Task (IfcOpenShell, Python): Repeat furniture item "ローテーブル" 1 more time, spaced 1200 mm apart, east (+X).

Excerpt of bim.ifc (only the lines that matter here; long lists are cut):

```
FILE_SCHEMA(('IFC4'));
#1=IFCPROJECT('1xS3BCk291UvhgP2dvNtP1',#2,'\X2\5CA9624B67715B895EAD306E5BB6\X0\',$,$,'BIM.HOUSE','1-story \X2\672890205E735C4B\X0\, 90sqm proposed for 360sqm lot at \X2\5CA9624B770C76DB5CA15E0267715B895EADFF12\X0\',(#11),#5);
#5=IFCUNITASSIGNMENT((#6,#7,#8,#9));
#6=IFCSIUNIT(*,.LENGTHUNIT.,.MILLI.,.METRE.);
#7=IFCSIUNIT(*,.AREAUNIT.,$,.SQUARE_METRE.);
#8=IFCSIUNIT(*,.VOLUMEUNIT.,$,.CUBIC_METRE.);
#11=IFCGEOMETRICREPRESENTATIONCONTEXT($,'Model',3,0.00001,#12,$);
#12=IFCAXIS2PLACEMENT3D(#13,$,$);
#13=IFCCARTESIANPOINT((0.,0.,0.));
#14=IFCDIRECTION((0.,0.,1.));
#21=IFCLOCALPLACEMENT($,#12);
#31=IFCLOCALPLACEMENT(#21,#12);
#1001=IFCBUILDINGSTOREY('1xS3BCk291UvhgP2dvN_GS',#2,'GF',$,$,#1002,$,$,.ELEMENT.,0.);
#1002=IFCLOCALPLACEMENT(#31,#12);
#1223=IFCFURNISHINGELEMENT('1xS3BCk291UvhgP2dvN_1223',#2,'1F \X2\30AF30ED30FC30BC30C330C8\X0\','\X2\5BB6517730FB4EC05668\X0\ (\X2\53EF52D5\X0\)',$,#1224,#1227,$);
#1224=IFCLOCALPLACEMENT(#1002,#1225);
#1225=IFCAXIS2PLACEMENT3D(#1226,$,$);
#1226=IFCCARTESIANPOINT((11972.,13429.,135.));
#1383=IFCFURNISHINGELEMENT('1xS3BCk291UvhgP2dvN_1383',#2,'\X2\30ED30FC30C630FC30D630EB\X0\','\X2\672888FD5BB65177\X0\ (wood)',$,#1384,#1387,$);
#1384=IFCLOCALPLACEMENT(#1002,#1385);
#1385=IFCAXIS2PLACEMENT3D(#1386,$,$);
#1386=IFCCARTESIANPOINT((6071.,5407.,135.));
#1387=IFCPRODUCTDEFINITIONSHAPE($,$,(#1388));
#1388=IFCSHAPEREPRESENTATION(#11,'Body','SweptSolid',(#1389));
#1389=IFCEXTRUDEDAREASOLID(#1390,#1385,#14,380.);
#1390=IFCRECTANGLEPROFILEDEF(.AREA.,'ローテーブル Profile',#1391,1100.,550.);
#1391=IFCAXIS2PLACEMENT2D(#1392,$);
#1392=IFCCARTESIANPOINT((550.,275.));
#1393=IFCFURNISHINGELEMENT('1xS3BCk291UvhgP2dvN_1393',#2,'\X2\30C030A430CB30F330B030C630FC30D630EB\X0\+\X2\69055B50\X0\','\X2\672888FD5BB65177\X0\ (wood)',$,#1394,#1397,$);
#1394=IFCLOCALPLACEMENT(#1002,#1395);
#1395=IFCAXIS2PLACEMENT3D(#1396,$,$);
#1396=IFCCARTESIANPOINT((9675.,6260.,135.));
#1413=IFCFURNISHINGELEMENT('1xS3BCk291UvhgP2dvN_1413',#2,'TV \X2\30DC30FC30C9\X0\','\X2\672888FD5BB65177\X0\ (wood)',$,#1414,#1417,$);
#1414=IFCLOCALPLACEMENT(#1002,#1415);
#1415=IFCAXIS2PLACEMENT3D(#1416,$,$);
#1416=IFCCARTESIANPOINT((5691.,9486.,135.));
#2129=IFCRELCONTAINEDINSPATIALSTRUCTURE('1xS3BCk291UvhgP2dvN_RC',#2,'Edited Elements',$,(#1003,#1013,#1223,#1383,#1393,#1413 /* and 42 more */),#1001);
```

```python
import numpy as np
import ifcopenshell
import ifcopenshell.api.geometry
import ifcopenshell.api.root
import ifcopenshell.util.element
import ifcopenshell.util.placement
import ifcopenshell.util.unit

model = ifcopenshell.open("bim.ifc")
unit_scale = ifcopenshell.util.unit.calculate_unit_scale(model)


def reuse_history(source, copy):
    """copy_class also copies each property set's owner history, people and application; keep the originals."""
    for rel in copy.IsDefinedBy:
        if rel.is_a("IfcRelDefinesByProperties") and (history := rel.RelatingPropertyDefinition.OwnerHistory):
            rel.RelatingPropertyDefinition.OwnerHistory = source.OwnerHistory
            ifcopenshell.util.element.remove_deep2(model, history)


source = model.by_guid("1xS3BCk291UvhgP2dvN_1383")
base = ifcopenshell.util.placement.get_local_placement(source.ObjectPlacement)
step = np.array([1.0, 0.0, 0.0]) * 1.2 / unit_scale

for i in range(1, 2):
    copy = ifcopenshell.api.root.copy_class(model, product=source)
    copy.Representation = ifcopenshell.util.element.copy_deep(
        model, source.Representation, exclude=["IfcGeometricRepresentationContext", "IfcRepresentationMap"]
    )
    reuse_history(source, copy)
    matrix = base.copy()
    matrix[:3, 3] += i * step
    print("added at", matrix[:3, 3].round(3) + 0.0)
    ifcopenshell.api.geometry.edit_object_placement(model, product=copy, matrix=matrix, is_si=False)

model.write("bim_v2.ifc")
```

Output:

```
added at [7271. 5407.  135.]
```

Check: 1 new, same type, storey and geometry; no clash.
